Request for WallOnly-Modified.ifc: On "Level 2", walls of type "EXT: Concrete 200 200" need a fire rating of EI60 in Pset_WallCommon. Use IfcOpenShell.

First a look at what the model holds.

```python
import ifcopenshell
import ifcopenshell.util.element

model = ifcopenshell.open("WallOnly-Modified.ifc")
print(model.schema)
storey = next(s for s in model.by_type("IfcBuildingStorey") if s.Name == "Level 2")
walls = [e for e in ifcopenshell.util.element.get_decomposition(storey) if e.is_a("IfcWall")]
seen = {}
for e in walls:
    element_type = ifcopenshell.util.element.get_type(e)
    key = (element_type.Name if element_type != e and element_type else None, ifcopenshell.util.element.get_pset(e, "Pset_WallCommon", "FireRating"))
    seen[key] = seen.get(key, 0) + 1
for (name, value), count in sorted(seen.items(), key=str):
    print(count, "x", name, "|", value)
```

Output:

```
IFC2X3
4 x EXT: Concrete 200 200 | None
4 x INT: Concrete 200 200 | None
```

```python
import ifcopenshell
import ifcopenshell.api.pset
import ifcopenshell.util.element

model = ifcopenshell.open("WallOnly-Modified.ifc")

storey = next(s for s in model.by_type("IfcBuildingStorey") if s.Name == "Level 2")
walls = [e for e in ifcopenshell.util.element.get_decomposition(storey) if e.is_a("IfcWall")]

count = 0
for e in walls:
    element_type = ifcopenshell.util.element.get_type(e)
    if element_type in (None, e) or element_type.Name != "EXT: Concrete 200 200":
        continue
    # add_pset returns the element's existing set when there is one.
    pset = ifcopenshell.api.pset.add_pset(model, product=e, name="Pset_WallCommon")
    ifcopenshell.api.pset.edit_pset(model, pset=pset, properties={"FireRating": "EI60"})
    count += 1

print(count, "walls updated")

model.write("WallOnly-Modified_v2.ifc")
```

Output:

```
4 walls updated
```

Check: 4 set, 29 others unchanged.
